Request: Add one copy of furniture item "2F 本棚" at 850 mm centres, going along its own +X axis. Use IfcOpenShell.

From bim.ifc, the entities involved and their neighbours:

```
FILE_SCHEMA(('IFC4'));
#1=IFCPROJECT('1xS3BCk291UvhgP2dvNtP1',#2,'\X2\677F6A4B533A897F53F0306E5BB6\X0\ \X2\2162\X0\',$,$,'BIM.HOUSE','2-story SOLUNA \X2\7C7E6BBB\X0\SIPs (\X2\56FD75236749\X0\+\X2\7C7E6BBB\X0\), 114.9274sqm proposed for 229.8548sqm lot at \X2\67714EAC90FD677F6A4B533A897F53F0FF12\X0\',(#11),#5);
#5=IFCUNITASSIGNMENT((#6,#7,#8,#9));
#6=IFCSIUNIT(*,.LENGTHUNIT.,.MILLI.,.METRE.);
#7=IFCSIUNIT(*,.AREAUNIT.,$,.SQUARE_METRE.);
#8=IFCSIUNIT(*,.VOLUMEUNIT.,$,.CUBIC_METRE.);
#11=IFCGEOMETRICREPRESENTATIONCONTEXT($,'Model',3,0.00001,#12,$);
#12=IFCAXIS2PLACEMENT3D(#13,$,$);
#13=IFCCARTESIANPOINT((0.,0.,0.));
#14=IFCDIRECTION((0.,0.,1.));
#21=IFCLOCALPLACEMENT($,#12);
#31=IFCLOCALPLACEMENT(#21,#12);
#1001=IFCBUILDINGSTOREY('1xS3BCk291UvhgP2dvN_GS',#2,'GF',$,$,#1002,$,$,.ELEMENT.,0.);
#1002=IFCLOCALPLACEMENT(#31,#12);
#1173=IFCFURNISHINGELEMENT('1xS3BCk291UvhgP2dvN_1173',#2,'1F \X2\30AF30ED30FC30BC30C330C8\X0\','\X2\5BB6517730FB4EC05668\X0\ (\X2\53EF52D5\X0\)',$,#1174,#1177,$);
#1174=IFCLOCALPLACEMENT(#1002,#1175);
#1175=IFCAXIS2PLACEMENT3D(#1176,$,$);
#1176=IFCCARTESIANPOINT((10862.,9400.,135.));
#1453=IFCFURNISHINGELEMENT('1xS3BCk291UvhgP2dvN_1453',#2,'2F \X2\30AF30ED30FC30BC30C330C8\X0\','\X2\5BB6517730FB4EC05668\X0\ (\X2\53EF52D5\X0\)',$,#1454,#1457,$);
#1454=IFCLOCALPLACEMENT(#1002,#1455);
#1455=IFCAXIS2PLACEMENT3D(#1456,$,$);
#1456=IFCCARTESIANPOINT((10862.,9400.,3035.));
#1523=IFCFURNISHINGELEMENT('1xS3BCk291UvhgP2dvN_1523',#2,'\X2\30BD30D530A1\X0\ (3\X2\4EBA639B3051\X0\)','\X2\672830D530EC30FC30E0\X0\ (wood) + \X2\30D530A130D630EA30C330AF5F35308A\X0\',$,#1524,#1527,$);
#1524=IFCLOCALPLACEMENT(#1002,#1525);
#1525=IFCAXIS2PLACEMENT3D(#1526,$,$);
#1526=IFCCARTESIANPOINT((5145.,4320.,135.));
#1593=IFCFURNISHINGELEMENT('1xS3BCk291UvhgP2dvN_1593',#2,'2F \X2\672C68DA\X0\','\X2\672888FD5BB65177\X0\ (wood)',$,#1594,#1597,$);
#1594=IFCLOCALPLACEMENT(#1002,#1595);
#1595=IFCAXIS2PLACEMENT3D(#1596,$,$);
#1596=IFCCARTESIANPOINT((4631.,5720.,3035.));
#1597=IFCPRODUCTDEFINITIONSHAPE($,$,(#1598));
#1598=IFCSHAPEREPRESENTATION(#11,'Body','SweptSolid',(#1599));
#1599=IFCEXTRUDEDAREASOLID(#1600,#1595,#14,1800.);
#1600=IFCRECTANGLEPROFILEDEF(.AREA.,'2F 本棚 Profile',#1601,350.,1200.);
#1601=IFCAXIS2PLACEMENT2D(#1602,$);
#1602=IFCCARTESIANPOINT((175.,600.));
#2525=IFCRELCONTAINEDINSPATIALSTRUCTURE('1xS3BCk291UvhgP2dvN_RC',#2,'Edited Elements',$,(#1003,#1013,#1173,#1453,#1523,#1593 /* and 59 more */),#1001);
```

```python
import ifcopenshell
import ifcopenshell.api.geometry
import ifcopenshell.api.root
import ifcopenshell.util.element
import ifcopenshell.util.placement

model = ifcopenshell.open("bim.ifc")


def reuse_history(source, copy):
    """copy_class also copies each property set's owner history, people and application; keep the originals."""
    for rel in copy.IsDefinedBy:
        if rel.is_a("IfcRelDefinesByProperties") and (history := rel.RelatingPropertyDefinition.OwnerHistory):
            rel.RelatingPropertyDefinition.OwnerHistory = source.OwnerHistory
            ifcopenshell.util.element.remove_deep2(model, history)


source = model.by_id(1593)
base = ifcopenshell.util.placement.get_local_placement(source.ObjectPlacement)
step = base[:3, 0] * 850.0

for i in range(1, 2):
    copy = ifcopenshell.api.root.copy_class(model, product=source)
    copy.Representation = ifcopenshell.util.element.copy_deep(
        model, source.Representation, exclude=["IfcGeometricRepresentationContext", "IfcRepresentationMap"]
    )
    reuse_history(source, copy)
    matrix = base.copy()
    matrix[:3, 3] += i * step
    print("added at", matrix[:3, 3].round(3) + 0.0)
    ifcopenshell.api.geometry.edit_object_placement(model, product=copy, matrix=matrix, is_si=False)

model.write("bim-out.ifc")
```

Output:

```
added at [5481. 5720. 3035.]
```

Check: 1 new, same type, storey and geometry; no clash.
